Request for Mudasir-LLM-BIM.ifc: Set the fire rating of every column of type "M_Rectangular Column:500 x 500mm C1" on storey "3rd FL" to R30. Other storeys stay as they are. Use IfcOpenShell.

First a look at what the model holds.

```python
import ifcopenshell
import ifcopenshell.util.element

model = ifcopenshell.open("Mudasir-LLM-BIM.ifc")
print(model.schema)
storey = next(s for s in model.by_type("IfcBuildingStorey") if s.Name == "3rd FL")
columns = [e for e in ifcopenshell.util.element.get_decomposition(storey) if e.is_a("IfcColumn")]
seen = {}
for e in columns:
    element_type = ifcopenshell.util.element.get_type(e)
    key = (element_type.Name if element_type != e and element_type else None, ifcopenshell.util.element.get_pset(e, "Pset_ColumnCommon", "FireRating"))
    seen[key] = seen.get(key, 0) + 1
for (name, value), count in sorted(seen.items(), key=str):
    print(count, "x", name, "|", value)
```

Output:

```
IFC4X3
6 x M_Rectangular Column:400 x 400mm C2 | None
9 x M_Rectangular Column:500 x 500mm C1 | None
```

```python
import ifcopenshell
import ifcopenshell.api.pset
import ifcopenshell.util.element

model = ifcopenshell.open("Mudasir-LLM-BIM.ifc")

storey = next(s for s in model.by_type("IfcBuildingStorey") if s.Name == "3rd FL")
columns = [e for e in ifcopenshell.util.element.get_decomposition(storey) if e.is_a("IfcColumn")]

count = 0
for e in columns:
    element_type = ifcopenshell.util.element.get_type(e)
    if element_type in (None, e) or element_type.Name != "M_Rectangular Column:500 x 500mm C1":
        continue
    # add_pset returns the element's existing set when there is one.
    pset = ifcopenshell.api.pset.add_pset(model, product=e, name="Pset_ColumnCommon")
    ifcopenshell.api.pset.edit_pset(model, pset=pset, properties={"FireRating": "R30"})
    count += 1

print(count, "columns updated")

model.write("Mudasir-LLM-BIM-out.ifc")
```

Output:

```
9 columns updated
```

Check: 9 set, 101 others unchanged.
